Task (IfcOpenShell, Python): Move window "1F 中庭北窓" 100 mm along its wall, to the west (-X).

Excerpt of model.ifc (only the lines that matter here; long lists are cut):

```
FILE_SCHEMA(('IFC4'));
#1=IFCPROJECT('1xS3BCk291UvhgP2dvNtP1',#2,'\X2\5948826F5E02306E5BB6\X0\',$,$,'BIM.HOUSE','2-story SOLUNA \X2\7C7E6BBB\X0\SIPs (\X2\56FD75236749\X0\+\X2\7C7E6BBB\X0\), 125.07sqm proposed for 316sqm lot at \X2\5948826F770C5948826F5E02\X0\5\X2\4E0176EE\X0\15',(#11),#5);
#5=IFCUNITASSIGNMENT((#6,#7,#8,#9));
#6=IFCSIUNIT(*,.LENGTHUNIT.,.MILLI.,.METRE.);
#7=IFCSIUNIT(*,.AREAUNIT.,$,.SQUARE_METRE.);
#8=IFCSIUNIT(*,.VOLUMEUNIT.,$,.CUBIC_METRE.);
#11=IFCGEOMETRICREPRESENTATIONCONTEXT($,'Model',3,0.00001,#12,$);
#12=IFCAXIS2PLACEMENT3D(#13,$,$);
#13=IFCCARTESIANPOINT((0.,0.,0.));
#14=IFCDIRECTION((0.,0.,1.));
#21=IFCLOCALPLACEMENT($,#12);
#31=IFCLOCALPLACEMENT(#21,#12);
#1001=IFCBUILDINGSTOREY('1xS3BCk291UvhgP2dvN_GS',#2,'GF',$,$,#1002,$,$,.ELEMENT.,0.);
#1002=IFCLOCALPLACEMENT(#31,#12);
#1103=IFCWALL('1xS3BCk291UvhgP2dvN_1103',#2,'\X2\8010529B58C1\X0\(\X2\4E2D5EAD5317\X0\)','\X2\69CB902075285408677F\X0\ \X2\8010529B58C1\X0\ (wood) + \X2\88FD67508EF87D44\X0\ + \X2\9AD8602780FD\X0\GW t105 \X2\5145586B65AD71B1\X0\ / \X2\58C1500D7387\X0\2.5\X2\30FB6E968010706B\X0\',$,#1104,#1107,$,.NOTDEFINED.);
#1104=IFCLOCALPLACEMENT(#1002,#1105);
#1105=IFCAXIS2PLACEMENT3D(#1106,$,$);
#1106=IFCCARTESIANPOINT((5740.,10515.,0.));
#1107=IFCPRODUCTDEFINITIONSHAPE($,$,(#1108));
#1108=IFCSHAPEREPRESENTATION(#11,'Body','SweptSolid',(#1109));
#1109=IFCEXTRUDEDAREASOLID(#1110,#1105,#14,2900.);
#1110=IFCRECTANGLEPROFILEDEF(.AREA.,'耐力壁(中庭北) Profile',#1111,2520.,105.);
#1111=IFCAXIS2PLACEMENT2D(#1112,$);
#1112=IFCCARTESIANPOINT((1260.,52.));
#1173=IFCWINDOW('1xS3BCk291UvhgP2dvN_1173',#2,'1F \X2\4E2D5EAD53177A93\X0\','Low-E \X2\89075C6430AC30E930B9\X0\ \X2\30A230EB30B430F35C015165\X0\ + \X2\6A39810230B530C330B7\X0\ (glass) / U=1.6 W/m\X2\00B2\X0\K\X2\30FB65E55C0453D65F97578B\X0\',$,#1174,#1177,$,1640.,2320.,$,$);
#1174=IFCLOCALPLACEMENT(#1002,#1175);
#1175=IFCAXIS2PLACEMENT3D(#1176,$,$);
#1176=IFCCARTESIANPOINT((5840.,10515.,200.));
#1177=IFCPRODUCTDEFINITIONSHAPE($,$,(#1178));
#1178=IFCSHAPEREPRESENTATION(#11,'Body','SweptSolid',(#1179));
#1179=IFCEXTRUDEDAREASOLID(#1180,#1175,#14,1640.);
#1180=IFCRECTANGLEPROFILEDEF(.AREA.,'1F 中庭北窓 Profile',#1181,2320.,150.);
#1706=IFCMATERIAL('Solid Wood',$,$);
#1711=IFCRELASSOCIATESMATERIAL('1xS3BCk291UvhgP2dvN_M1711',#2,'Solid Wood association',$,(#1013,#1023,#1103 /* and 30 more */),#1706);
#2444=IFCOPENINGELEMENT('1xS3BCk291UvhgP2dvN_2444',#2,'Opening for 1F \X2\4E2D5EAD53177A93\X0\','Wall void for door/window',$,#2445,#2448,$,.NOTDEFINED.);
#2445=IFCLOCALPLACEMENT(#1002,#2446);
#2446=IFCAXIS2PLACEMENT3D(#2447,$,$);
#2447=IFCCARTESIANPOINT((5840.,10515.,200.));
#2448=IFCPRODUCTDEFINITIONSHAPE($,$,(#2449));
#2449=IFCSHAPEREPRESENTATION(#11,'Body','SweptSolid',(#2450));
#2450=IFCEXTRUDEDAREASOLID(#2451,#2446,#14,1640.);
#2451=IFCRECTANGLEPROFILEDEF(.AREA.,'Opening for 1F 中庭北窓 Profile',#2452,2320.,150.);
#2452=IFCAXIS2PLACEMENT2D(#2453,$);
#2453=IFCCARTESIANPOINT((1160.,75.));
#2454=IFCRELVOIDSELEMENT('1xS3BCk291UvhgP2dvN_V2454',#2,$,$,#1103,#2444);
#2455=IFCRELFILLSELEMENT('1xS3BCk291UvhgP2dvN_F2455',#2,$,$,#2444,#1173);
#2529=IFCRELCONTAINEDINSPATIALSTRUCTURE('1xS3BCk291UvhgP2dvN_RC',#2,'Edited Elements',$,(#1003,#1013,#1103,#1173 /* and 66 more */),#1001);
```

```python
import ifcopenshell
import ifcopenshell.api.geometry
import ifcopenshell.util.placement

model = ifcopenshell.open("model.ifc")

window = model.by_id(1173)
opening = window.FillsVoids[0].RelatingOpeningElement
wall = opening.VoidsElements[0].RelatingBuildingElement

wall_matrix = ifcopenshell.util.placement.get_local_placement(wall.ObjectPlacement)
shift = wall_matrix[:3, 0] * -100.0
before = ifcopenshell.util.placement.get_local_placement(window.ObjectPlacement)[:3, 3].copy()

# The window is not placed relative to its opening, so move both.
for product in (opening, window):
    matrix = ifcopenshell.util.placement.get_local_placement(product.ObjectPlacement)
    matrix[:3, 3] += shift
    ifcopenshell.api.geometry.edit_object_placement(model, product=product, matrix=matrix, is_si=False)

after = ifcopenshell.util.placement.get_local_placement(window.ObjectPlacement)[:3, 3]
print("window moved by", (after - before).round(3) + 0.0)

model.write("model-out.ifc")
```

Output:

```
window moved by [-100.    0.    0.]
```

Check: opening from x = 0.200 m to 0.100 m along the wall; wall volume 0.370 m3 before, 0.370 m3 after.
